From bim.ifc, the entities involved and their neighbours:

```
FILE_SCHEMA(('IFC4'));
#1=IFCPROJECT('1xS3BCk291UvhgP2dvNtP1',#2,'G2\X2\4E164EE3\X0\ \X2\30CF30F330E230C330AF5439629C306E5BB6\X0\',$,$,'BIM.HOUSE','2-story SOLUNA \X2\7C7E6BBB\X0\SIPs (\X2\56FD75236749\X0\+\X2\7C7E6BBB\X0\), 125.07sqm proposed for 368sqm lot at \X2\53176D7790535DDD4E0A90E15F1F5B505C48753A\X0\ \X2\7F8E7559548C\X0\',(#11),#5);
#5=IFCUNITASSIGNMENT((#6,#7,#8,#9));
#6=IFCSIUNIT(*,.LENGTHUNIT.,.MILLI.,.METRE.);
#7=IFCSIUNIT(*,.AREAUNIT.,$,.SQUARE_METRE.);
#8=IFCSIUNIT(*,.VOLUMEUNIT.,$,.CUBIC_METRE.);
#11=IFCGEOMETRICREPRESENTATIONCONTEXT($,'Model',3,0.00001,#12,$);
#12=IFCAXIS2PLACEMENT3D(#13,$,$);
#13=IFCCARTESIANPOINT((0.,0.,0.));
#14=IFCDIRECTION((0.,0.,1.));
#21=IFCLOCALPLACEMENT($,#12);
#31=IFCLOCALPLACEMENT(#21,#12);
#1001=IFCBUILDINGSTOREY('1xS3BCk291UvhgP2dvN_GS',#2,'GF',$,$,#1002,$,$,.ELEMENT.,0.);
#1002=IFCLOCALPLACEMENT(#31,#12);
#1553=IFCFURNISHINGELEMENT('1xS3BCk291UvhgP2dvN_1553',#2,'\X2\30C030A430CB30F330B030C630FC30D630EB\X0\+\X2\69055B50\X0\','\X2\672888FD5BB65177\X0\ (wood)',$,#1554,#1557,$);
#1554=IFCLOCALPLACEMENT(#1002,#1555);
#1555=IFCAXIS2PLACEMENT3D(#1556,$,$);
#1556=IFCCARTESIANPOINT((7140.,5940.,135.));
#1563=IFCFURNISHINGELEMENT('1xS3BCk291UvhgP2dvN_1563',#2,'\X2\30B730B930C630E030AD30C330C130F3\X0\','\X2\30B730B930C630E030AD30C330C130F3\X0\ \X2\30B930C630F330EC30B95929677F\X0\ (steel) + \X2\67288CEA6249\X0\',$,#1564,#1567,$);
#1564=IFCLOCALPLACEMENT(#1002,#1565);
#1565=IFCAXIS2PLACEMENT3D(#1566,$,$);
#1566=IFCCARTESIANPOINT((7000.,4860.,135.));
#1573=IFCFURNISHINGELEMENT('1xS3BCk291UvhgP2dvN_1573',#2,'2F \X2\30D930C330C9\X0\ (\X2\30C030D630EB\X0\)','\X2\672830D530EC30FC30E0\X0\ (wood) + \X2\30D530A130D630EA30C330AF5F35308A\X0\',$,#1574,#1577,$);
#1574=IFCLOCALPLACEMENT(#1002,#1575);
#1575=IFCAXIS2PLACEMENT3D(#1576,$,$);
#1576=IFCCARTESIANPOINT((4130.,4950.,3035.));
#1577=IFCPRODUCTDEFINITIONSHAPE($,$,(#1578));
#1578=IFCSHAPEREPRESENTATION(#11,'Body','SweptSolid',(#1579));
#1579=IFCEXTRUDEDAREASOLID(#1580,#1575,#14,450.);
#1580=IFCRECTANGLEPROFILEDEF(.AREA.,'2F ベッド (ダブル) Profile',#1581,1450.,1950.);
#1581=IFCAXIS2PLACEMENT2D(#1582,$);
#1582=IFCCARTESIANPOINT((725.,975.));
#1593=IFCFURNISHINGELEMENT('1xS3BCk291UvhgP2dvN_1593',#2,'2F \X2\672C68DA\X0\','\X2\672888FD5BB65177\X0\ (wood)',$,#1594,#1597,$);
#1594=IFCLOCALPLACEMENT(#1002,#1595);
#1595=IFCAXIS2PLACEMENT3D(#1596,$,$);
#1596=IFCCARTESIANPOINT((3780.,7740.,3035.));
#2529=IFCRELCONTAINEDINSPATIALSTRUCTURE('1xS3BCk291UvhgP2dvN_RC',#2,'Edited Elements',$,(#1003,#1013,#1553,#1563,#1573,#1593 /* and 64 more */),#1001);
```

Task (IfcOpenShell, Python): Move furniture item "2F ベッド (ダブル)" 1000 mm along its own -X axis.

```python
import ifcopenshell
import ifcopenshell.api.geometry
import ifcopenshell.util.placement
import ifcopenshell.util.unit

model = ifcopenshell.open("bim.ifc")
unit_scale = ifcopenshell.util.unit.calculate_unit_scale(model)

item = model.by_id(1573)
matrix = ifcopenshell.util.placement.get_local_placement(item.ObjectPlacement)
matrix[:3, 3] -= matrix[:3, 0] * 1 / unit_scale
ifcopenshell.api.geometry.edit_object_placement(model, product=item, matrix=matrix, is_si=False)

print(ifcopenshell.util.placement.get_local_placement(item.ObjectPlacement).round(3) + 0.0)

model.write("bim_v2.ifc")
```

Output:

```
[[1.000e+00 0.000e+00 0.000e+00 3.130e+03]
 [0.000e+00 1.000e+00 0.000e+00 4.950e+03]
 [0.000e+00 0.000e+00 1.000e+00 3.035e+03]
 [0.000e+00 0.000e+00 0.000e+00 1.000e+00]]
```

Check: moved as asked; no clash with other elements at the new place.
